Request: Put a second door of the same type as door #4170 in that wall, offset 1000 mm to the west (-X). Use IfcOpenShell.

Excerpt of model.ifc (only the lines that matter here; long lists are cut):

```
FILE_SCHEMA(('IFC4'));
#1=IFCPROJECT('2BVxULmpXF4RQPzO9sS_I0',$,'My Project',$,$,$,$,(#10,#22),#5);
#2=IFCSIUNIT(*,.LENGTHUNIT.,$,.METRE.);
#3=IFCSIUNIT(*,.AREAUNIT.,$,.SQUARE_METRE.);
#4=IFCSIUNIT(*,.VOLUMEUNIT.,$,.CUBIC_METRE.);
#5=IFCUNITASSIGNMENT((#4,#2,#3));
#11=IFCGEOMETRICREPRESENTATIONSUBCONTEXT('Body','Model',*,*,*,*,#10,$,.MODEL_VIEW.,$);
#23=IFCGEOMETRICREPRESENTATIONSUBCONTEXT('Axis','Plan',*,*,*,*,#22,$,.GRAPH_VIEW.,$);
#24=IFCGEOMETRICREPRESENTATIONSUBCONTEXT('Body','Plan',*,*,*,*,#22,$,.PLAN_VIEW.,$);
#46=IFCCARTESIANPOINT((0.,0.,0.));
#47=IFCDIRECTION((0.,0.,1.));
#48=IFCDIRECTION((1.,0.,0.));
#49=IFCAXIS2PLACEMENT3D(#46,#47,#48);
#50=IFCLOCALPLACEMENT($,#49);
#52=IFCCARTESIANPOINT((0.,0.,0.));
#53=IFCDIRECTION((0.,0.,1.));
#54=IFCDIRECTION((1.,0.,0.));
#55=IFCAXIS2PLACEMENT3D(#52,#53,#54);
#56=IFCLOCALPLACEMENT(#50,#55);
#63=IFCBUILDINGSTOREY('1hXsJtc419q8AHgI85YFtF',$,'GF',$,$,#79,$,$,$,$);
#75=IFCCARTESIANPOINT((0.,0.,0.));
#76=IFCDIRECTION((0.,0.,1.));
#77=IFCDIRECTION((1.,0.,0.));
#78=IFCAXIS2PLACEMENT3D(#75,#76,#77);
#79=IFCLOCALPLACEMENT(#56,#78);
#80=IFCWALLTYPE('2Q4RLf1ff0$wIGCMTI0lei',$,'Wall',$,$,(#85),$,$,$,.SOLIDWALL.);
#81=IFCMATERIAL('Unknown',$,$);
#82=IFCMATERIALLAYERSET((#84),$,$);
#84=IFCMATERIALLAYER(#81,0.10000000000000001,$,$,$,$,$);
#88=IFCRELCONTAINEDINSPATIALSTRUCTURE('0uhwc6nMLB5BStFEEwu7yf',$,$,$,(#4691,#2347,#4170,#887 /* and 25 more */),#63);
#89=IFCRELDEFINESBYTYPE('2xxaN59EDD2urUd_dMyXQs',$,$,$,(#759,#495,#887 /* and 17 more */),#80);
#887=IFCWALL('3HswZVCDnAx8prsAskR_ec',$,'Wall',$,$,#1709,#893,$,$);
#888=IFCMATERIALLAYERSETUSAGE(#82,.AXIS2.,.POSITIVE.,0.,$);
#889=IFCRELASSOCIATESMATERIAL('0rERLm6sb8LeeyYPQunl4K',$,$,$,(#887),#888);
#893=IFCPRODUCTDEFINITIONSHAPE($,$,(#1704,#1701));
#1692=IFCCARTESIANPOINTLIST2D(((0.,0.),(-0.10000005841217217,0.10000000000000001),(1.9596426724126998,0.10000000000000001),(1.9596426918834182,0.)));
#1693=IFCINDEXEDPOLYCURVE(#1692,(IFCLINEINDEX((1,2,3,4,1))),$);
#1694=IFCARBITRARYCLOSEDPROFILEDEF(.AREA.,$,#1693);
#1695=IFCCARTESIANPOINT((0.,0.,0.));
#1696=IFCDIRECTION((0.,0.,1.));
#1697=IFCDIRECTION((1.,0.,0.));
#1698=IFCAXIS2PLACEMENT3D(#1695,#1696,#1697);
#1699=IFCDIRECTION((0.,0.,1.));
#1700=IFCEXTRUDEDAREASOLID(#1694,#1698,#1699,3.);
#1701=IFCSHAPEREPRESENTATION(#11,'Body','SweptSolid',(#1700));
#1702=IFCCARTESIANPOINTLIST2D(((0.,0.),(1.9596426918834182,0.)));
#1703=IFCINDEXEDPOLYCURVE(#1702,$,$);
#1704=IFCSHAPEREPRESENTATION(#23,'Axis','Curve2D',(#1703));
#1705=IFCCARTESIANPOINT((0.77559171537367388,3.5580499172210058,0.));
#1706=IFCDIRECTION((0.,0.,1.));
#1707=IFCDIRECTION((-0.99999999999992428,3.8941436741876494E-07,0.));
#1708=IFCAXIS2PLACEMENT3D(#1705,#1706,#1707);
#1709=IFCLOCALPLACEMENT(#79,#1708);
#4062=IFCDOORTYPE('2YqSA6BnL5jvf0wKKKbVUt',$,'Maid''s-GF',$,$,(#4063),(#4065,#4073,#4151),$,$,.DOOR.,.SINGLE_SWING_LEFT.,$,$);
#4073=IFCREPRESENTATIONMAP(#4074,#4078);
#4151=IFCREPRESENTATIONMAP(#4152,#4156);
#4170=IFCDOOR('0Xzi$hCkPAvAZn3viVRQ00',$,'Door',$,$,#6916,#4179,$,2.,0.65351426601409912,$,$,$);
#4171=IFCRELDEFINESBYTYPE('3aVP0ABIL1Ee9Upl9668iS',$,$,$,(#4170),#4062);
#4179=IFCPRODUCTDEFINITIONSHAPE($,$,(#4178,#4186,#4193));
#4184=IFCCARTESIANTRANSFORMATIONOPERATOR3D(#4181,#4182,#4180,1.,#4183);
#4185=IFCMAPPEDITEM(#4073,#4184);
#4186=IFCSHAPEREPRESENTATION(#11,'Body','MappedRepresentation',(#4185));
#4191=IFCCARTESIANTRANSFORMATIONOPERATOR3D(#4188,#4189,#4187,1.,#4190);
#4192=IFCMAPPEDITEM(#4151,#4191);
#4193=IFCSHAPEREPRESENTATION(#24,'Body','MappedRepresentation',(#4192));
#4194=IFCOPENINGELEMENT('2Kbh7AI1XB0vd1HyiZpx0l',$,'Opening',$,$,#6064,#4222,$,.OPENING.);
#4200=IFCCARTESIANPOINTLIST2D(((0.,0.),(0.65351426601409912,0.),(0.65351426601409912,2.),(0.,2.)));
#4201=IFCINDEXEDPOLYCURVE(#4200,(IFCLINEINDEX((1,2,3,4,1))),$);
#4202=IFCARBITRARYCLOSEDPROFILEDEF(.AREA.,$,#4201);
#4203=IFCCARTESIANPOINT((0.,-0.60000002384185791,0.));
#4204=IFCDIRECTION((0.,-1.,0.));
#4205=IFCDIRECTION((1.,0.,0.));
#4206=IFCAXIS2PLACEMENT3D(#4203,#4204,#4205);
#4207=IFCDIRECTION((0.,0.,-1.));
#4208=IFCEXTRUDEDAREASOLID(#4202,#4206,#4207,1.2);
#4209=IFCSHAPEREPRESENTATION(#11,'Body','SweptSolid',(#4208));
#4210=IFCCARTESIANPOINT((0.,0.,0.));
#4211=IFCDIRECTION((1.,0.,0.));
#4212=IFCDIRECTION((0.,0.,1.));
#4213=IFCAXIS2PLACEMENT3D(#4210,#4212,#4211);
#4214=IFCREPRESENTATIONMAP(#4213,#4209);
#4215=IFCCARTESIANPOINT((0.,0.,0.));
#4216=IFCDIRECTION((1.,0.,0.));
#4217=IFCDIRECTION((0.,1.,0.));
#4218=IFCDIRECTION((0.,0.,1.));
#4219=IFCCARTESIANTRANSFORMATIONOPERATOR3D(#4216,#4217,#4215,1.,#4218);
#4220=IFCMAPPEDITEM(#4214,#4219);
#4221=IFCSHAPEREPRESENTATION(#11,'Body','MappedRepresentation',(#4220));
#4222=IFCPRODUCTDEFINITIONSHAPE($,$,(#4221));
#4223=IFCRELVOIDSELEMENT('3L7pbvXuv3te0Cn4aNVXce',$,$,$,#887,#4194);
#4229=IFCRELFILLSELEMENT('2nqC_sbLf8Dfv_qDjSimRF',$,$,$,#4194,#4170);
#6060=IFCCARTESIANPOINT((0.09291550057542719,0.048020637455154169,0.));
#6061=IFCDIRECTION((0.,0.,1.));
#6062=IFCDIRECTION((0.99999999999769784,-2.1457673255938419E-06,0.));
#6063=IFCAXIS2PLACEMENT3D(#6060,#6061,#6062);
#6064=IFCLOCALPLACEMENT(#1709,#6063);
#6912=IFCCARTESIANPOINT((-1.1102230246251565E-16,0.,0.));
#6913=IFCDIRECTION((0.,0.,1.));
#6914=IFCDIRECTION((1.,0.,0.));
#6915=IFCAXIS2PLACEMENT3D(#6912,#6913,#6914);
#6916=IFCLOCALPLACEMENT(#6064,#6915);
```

```python
import ifcopenshell
import ifcopenshell.api.feature
import ifcopenshell.api.geometry
import ifcopenshell.api.root
import ifcopenshell.geom
import ifcopenshell.util.element
import ifcopenshell.util.placement
import ifcopenshell.util.shape
import ifcopenshell.util.unit

model = ifcopenshell.open("model.ifc")
unit_scale = ifcopenshell.util.unit.calculate_unit_scale(model)
settings = ifcopenshell.geom.settings()


def volume(element):
    """Net volume in cubic metres, openings subtracted."""
    shape = ifcopenshell.geom.create_shape(settings, element)
    return ifcopenshell.util.shape.get_volume(shape.geometry)


door = model.by_guid("0Xzi$hCkPAvAZn3viVRQ00")
opening = door.FillsVoids[0].RelatingOpeningElement
wall = opening.VoidsElements[0].RelatingBuildingElement
before = volume(wall)
shift = ifcopenshell.util.placement.get_local_placement(wall.ObjectPlacement)[:3, 0] * 1 / unit_scale

# copy_class copies the void relationship, type, container and properties, but no geometry.
new_opening = ifcopenshell.api.root.copy_class(model, product=opening)
new_opening.Representation = ifcopenshell.util.element.copy_deep(
    model, opening.Representation, exclude=["IfcGeometricRepresentationContext", "IfcRepresentationMap"]
)
new_door = ifcopenshell.api.root.copy_class(model, product=door)
new_door.Representation = ifcopenshell.util.element.copy_deep(
    model, door.Representation, exclude=["IfcGeometricRepresentationContext", "IfcRepresentationMap"]
)
ifcopenshell.api.feature.add_filling(model, opening=new_opening, element=new_door)

for old, new in ((opening, new_opening), (door, new_door)):
    matrix = ifcopenshell.util.placement.get_local_placement(old.ObjectPlacement)
    matrix[:3, 3] += shift
    ifcopenshell.api.geometry.edit_object_placement(model, product=new, matrix=matrix, is_si=False)

after = volume(wall)

print(f"wall volume {before:.3f} -> {after:.3f} m3")

model.write("model_rev.ifc")
```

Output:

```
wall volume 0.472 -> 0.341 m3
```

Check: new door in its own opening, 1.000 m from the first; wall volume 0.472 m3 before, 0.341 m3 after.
